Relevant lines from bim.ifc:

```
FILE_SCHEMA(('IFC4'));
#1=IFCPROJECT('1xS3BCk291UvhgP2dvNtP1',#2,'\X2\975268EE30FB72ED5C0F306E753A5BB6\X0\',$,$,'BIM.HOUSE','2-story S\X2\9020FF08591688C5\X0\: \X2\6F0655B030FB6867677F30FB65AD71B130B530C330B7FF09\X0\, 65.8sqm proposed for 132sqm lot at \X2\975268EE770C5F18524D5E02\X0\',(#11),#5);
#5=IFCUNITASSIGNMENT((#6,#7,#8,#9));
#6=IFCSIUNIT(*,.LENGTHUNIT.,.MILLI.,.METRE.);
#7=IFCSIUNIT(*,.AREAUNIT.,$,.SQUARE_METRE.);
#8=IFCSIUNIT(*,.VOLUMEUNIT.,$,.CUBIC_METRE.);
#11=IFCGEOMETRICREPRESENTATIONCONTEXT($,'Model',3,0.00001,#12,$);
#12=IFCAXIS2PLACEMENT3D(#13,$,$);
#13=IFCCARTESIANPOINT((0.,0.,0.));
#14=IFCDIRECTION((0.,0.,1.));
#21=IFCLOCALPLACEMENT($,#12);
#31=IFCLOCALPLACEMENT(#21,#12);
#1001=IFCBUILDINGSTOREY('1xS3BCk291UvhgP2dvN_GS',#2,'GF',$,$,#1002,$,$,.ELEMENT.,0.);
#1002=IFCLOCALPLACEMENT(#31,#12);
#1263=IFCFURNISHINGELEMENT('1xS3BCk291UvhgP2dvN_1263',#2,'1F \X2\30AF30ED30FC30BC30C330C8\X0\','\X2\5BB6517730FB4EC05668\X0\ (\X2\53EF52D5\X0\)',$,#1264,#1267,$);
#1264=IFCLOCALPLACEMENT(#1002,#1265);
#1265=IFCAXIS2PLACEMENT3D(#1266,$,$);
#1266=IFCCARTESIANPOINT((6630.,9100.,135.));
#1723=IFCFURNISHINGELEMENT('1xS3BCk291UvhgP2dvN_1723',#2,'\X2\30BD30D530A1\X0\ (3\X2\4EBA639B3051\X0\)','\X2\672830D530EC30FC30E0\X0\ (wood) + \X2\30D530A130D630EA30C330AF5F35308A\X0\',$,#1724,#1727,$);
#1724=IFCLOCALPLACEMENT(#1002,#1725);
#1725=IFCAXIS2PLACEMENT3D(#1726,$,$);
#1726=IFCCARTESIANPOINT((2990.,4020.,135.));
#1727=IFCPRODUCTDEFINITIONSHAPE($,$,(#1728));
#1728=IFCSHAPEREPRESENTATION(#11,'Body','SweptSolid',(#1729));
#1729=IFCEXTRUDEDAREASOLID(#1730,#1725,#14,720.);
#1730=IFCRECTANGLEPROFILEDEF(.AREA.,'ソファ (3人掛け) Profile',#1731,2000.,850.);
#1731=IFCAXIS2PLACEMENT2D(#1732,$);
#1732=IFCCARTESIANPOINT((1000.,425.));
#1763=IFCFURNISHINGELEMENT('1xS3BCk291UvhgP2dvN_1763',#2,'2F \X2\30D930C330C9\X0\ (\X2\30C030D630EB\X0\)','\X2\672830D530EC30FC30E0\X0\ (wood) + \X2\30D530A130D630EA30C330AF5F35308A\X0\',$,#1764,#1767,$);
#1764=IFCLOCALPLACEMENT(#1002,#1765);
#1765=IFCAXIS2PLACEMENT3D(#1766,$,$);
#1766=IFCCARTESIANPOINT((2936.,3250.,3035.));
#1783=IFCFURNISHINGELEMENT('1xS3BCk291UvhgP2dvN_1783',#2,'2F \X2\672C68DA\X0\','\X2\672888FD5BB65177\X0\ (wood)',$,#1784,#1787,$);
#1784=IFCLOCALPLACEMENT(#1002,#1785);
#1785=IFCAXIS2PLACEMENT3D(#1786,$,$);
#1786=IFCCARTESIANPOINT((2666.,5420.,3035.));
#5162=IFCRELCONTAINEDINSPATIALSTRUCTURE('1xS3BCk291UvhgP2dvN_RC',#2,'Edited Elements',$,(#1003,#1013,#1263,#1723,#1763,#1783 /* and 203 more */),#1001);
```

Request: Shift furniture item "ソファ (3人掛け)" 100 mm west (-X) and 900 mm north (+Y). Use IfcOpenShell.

```python
import ifcopenshell
import ifcopenshell.api.geometry
import ifcopenshell.util.placement
import ifcopenshell.util.unit

model = ifcopenshell.open("bim.ifc")
unit_scale = ifcopenshell.util.unit.calculate_unit_scale(model)

item = model.by_guid("1xS3BCk291UvhgP2dvN_1723")
matrix = ifcopenshell.util.placement.get_local_placement(item.ObjectPlacement)
matrix[0, 3] -= 0.1 / unit_scale
matrix[1, 3] += 0.9 / unit_scale
ifcopenshell.api.geometry.edit_object_placement(model, product=item, matrix=matrix, is_si=False)

print(ifcopenshell.util.placement.get_local_placement(item.ObjectPlacement).round(3) + 0.0)

model.write("bim_edited.ifc")
```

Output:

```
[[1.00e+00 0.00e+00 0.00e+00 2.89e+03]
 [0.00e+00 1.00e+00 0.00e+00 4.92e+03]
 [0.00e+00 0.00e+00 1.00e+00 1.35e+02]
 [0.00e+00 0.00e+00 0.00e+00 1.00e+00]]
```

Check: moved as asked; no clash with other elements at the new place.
